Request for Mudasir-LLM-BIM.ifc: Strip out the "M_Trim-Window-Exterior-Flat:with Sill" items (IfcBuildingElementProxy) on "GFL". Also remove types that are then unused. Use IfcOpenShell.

First a look at what the model holds.

```python
import ifcopenshell
import ifcopenshell.util.element

model = ifcopenshell.open("Mudasir-LLM-BIM.ifc")
print(model.schema)
storey = next(s for s in model.by_type("IfcBuildingStorey") if s.Name == "GFL")
proxies = [e for e in ifcopenshell.util.element.get_decomposition(storey) if e.is_a("IfcBuildingElementProxy")]
seen = {}
for e in proxies:
    element_type = ifcopenshell.util.element.get_type(e)
    name = element_type.Name if element_type not in (None, e) else None
    seen[name] = seen.get(name, 0) + 1
for name, count in sorted(seen.items(), key=str):
    print(count, "x", name)
```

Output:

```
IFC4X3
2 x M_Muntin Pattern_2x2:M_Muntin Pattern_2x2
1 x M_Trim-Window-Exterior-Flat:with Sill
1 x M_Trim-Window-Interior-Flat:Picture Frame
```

```python
import ifcopenshell
import ifcopenshell.api.root
import ifcopenshell.util.element

model = ifcopenshell.open("Mudasir-LLM-BIM.ifc")

storey = next(s for s in model.by_type("IfcBuildingStorey") if s.Name == "GFL")
proxies = [e for e in ifcopenshell.util.element.get_decomposition(storey) if e.is_a("IfcBuildingElementProxy")]
targets = [e for e in proxies if (t := ifcopenshell.util.element.get_type(e)) not in (None, e) and t.Name == "M_Trim-Window-Exterior-Flat:with Sill"]
types = {ifcopenshell.util.element.get_type(e) for e in targets} - {None, *targets}

for e in targets:
    ifcopenshell.api.root.remove_product(model, product=e)
print(len(targets), "removed")

unused = [t for t in types if not ifcopenshell.util.element.get_types(t)]
for t in unused:
    ifcopenshell.api.root.remove_product(model, product=t)
print(len(unused), "unused types removed")

model.write("Mudasir-LLM-BIM-out.ifc")
```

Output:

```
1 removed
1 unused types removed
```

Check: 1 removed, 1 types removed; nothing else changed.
